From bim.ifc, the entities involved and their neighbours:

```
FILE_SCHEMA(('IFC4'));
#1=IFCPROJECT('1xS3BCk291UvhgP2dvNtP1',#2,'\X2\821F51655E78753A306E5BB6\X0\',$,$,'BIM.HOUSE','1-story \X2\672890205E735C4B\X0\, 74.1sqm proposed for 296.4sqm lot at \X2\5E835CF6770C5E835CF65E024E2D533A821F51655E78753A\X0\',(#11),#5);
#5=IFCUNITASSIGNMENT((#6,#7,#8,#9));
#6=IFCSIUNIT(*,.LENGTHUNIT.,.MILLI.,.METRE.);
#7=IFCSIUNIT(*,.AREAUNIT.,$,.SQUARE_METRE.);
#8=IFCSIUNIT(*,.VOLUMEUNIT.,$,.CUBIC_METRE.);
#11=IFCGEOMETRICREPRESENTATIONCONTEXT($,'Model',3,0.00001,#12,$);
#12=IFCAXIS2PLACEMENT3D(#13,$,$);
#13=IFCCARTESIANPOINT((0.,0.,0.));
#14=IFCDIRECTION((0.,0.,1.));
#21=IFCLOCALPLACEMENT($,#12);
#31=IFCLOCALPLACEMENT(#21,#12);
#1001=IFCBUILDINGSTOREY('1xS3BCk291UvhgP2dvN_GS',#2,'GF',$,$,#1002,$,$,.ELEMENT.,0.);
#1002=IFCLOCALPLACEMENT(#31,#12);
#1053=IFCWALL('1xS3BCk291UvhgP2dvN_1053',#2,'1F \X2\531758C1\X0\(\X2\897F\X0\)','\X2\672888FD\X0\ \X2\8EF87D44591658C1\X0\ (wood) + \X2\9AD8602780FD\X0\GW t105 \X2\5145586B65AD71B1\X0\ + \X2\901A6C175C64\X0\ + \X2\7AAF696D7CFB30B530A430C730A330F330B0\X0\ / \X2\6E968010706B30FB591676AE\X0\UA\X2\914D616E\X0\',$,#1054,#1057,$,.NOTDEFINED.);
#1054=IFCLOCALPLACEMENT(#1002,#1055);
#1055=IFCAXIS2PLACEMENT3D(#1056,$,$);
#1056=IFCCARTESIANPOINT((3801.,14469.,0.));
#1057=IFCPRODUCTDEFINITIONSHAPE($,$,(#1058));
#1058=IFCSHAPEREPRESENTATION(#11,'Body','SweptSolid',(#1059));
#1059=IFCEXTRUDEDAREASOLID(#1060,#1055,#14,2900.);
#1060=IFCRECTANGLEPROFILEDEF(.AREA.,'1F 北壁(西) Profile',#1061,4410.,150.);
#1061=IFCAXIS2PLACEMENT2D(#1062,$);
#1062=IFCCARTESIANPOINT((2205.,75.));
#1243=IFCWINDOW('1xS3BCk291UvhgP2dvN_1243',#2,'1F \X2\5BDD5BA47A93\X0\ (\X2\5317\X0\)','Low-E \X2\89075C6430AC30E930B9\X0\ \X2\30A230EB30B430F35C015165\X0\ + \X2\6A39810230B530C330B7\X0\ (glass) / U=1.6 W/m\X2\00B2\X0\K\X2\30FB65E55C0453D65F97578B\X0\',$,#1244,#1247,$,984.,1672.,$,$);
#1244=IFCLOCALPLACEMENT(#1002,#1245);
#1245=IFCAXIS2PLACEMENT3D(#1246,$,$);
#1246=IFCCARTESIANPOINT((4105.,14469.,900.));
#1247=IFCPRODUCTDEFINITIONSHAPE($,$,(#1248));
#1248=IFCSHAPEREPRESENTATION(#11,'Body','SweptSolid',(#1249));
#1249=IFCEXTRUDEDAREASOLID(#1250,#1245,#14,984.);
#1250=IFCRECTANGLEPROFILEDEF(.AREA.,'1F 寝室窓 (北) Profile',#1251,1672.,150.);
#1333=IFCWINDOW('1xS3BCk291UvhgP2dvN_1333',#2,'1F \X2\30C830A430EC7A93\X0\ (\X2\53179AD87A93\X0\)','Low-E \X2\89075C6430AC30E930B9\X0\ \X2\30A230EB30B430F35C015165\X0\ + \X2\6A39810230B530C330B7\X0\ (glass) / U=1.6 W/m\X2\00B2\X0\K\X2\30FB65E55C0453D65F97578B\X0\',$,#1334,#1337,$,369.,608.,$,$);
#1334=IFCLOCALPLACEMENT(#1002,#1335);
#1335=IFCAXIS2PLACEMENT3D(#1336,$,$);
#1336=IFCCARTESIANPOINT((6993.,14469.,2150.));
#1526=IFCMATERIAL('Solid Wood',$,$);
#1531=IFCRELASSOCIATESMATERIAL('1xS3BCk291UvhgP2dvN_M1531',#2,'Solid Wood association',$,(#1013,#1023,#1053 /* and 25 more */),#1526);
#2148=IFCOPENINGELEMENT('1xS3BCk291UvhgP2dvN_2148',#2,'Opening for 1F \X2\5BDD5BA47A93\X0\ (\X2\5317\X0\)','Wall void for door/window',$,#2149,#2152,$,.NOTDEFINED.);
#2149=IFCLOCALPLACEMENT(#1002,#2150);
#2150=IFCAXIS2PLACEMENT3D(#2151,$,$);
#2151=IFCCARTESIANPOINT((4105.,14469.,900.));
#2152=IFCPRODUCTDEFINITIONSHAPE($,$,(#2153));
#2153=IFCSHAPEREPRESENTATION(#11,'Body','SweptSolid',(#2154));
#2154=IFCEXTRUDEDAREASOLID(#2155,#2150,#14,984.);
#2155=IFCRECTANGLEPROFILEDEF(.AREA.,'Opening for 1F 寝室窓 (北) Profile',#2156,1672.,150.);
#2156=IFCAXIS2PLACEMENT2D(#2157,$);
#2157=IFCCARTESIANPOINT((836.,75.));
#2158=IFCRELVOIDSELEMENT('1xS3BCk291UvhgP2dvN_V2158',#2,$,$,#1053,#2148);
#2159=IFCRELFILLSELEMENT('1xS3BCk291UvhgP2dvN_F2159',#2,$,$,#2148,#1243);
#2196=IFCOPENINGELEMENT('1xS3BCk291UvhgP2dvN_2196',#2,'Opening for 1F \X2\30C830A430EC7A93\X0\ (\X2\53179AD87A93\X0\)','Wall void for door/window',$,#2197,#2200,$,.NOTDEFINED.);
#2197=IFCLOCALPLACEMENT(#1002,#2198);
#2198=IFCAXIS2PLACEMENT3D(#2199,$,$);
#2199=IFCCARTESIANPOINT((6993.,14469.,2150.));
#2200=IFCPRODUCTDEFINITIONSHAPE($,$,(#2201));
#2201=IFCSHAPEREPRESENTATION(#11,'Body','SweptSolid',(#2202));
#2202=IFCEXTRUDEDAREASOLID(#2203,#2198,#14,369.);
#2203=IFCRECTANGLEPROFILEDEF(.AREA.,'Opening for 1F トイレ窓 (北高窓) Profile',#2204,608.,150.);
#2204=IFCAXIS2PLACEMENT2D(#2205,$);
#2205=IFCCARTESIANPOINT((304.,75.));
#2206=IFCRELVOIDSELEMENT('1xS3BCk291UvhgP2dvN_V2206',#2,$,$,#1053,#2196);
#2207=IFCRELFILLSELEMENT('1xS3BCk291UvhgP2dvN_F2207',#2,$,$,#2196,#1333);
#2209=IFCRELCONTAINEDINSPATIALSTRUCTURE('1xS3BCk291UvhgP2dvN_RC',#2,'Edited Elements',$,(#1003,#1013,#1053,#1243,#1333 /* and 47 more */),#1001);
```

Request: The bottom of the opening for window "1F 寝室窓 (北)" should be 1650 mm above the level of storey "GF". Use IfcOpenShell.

```python
import numpy as np
import ifcopenshell
import ifcopenshell.api.geometry
import ifcopenshell.geom
import ifcopenshell.util.element
import ifcopenshell.util.placement
import ifcopenshell.util.shape
import ifcopenshell.util.unit

model = ifcopenshell.open("bim.ifc")
unit_scale = ifcopenshell.util.unit.calculate_unit_scale(model)

window = model.by_guid("1xS3BCk291UvhgP2dvN_1243")
opening = window.FillsVoids[0].RelatingOpeningElement
storey = ifcopenshell.util.element.get_container(window, ifc_class="IfcBuildingStorey")
level = ifcopenshell.util.placement.get_local_placement(storey.ObjectPlacement)[2, 3]

# The opening's origin need not be at the sill, so measure its lowest point.
shape = ifcopenshell.geom.create_shape(ifcopenshell.geom.settings(), opening)
bottom = ifcopenshell.util.shape.get_shape_bottom_elevation(shape, shape.geometry) / unit_scale
dz = level + 1.65 / unit_scale - bottom

shift = np.array([0.0, 0.0, dz])
# The window is not placed relative to its opening, so move both.
for product in (opening, window):
    matrix = ifcopenshell.util.placement.get_local_placement(product.ObjectPlacement)
    matrix[:3, 3] += shift
    ifcopenshell.api.geometry.edit_object_placement(model, product=product, matrix=matrix, is_si=False)

print(f"moved by {dz * unit_scale:+.3f} m")

model.write("bim_v2.ifc")
```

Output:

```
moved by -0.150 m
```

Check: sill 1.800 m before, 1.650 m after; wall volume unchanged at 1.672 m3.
